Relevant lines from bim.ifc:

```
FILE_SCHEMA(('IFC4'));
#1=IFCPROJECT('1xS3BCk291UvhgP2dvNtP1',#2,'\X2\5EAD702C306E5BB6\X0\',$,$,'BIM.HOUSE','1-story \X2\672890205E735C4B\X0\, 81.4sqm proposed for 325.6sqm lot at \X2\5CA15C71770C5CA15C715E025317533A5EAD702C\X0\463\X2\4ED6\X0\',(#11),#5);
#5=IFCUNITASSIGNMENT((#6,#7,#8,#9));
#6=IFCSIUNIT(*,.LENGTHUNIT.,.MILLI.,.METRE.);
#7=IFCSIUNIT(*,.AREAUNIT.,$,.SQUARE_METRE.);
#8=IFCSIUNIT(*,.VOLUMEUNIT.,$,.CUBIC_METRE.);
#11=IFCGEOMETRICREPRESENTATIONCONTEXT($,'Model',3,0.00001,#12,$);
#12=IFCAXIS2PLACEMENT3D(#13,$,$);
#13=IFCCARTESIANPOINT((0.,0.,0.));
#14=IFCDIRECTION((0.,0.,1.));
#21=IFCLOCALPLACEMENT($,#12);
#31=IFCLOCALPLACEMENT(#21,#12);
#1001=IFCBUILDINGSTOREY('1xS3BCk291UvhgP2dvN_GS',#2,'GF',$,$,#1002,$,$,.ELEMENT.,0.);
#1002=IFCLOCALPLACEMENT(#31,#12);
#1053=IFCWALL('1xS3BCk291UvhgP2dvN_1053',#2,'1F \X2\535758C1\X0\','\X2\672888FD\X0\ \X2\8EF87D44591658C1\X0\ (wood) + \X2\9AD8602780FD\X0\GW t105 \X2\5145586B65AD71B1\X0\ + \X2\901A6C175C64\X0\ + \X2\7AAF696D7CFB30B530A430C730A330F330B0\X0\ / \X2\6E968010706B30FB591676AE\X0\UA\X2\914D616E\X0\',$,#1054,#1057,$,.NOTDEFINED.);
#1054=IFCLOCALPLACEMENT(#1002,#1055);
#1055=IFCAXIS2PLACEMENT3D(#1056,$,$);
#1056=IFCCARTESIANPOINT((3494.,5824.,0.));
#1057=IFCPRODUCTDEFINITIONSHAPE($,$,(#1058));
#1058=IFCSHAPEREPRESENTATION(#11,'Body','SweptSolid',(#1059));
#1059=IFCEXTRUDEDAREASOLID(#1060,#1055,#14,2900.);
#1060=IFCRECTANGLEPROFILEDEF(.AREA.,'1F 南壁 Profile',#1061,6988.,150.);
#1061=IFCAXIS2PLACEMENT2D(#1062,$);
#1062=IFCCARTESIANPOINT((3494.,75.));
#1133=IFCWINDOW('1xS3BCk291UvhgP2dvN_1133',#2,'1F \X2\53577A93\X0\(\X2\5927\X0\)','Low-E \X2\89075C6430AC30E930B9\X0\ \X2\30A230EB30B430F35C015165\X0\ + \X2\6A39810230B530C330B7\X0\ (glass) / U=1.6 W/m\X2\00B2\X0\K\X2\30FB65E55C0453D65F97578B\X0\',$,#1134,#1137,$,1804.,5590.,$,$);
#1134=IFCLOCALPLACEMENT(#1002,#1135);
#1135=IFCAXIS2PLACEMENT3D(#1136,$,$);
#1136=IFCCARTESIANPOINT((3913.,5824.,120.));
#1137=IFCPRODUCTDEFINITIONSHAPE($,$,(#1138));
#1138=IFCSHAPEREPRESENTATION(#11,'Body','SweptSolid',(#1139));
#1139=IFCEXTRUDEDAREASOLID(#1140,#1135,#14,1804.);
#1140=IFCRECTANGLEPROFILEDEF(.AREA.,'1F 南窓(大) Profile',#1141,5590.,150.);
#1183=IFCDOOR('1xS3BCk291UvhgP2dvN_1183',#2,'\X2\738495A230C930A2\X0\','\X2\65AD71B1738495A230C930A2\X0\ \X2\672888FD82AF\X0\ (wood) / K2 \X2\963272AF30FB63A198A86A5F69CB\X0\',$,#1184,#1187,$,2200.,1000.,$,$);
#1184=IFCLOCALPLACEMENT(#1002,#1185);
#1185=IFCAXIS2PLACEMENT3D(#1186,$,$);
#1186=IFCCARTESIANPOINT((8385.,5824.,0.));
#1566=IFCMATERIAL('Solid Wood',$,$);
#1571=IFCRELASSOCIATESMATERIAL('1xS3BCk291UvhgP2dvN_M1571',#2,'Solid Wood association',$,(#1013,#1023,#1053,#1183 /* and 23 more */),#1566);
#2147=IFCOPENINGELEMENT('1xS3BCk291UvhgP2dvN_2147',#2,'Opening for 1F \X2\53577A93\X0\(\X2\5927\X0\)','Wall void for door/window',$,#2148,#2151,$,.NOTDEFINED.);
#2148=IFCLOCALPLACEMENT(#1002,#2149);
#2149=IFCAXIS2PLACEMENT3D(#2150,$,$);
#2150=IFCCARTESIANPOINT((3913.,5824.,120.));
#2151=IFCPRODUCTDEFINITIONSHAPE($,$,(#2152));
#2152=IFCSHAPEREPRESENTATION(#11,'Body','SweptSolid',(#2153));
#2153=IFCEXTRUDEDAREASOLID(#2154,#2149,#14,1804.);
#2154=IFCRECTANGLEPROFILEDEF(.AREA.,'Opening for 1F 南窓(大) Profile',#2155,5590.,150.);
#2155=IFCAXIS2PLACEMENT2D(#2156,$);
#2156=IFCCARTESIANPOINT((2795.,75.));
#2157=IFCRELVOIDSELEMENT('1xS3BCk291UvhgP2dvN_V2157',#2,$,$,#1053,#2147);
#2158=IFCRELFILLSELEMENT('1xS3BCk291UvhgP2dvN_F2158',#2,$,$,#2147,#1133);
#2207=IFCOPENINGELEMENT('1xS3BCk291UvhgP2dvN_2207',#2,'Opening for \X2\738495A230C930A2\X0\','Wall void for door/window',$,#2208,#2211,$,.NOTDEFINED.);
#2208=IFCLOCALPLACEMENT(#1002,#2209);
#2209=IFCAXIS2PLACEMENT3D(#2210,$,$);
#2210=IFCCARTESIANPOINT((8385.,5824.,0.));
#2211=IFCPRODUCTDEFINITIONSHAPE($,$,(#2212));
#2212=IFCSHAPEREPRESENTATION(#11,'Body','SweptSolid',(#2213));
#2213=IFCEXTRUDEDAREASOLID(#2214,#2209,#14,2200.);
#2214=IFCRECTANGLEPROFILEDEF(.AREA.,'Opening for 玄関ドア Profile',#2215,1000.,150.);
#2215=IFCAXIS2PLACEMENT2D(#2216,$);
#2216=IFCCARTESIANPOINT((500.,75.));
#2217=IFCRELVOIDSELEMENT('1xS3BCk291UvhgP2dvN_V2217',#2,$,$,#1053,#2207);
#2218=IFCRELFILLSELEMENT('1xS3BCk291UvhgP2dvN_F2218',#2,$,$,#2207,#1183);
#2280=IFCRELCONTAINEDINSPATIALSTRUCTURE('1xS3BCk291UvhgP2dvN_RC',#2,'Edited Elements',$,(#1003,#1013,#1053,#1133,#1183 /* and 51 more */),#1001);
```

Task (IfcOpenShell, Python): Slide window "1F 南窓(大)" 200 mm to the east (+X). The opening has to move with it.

```python
import ifcopenshell
import ifcopenshell.api.geometry
import ifcopenshell.util.placement
import ifcopenshell.util.unit

model = ifcopenshell.open("bim.ifc")
unit_scale = ifcopenshell.util.unit.calculate_unit_scale(model)

window = model.by_guid("1xS3BCk291UvhgP2dvN_1133")
opening = window.FillsVoids[0].RelatingOpeningElement
wall = opening.VoidsElements[0].RelatingBuildingElement

wall_matrix = ifcopenshell.util.placement.get_local_placement(wall.ObjectPlacement)
shift = wall_matrix[:3, 0] * 0.2 / unit_scale
before = ifcopenshell.util.placement.get_local_placement(window.ObjectPlacement)[:3, 3].copy()

# The window is not placed relative to its opening, so move both.
for product in (opening, window):
    matrix = ifcopenshell.util.placement.get_local_placement(product.ObjectPlacement)
    matrix[:3, 3] += shift
    ifcopenshell.api.geometry.edit_object_placement(model, product=product, matrix=matrix, is_si=False)

after = ifcopenshell.util.placement.get_local_placement(window.ObjectPlacement)[:3, 3]
print("window moved by", (after - before).round(3) + 0.0)

model.write("bim_edited.ifc")
```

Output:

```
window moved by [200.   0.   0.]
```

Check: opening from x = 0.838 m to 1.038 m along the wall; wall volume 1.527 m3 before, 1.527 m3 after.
